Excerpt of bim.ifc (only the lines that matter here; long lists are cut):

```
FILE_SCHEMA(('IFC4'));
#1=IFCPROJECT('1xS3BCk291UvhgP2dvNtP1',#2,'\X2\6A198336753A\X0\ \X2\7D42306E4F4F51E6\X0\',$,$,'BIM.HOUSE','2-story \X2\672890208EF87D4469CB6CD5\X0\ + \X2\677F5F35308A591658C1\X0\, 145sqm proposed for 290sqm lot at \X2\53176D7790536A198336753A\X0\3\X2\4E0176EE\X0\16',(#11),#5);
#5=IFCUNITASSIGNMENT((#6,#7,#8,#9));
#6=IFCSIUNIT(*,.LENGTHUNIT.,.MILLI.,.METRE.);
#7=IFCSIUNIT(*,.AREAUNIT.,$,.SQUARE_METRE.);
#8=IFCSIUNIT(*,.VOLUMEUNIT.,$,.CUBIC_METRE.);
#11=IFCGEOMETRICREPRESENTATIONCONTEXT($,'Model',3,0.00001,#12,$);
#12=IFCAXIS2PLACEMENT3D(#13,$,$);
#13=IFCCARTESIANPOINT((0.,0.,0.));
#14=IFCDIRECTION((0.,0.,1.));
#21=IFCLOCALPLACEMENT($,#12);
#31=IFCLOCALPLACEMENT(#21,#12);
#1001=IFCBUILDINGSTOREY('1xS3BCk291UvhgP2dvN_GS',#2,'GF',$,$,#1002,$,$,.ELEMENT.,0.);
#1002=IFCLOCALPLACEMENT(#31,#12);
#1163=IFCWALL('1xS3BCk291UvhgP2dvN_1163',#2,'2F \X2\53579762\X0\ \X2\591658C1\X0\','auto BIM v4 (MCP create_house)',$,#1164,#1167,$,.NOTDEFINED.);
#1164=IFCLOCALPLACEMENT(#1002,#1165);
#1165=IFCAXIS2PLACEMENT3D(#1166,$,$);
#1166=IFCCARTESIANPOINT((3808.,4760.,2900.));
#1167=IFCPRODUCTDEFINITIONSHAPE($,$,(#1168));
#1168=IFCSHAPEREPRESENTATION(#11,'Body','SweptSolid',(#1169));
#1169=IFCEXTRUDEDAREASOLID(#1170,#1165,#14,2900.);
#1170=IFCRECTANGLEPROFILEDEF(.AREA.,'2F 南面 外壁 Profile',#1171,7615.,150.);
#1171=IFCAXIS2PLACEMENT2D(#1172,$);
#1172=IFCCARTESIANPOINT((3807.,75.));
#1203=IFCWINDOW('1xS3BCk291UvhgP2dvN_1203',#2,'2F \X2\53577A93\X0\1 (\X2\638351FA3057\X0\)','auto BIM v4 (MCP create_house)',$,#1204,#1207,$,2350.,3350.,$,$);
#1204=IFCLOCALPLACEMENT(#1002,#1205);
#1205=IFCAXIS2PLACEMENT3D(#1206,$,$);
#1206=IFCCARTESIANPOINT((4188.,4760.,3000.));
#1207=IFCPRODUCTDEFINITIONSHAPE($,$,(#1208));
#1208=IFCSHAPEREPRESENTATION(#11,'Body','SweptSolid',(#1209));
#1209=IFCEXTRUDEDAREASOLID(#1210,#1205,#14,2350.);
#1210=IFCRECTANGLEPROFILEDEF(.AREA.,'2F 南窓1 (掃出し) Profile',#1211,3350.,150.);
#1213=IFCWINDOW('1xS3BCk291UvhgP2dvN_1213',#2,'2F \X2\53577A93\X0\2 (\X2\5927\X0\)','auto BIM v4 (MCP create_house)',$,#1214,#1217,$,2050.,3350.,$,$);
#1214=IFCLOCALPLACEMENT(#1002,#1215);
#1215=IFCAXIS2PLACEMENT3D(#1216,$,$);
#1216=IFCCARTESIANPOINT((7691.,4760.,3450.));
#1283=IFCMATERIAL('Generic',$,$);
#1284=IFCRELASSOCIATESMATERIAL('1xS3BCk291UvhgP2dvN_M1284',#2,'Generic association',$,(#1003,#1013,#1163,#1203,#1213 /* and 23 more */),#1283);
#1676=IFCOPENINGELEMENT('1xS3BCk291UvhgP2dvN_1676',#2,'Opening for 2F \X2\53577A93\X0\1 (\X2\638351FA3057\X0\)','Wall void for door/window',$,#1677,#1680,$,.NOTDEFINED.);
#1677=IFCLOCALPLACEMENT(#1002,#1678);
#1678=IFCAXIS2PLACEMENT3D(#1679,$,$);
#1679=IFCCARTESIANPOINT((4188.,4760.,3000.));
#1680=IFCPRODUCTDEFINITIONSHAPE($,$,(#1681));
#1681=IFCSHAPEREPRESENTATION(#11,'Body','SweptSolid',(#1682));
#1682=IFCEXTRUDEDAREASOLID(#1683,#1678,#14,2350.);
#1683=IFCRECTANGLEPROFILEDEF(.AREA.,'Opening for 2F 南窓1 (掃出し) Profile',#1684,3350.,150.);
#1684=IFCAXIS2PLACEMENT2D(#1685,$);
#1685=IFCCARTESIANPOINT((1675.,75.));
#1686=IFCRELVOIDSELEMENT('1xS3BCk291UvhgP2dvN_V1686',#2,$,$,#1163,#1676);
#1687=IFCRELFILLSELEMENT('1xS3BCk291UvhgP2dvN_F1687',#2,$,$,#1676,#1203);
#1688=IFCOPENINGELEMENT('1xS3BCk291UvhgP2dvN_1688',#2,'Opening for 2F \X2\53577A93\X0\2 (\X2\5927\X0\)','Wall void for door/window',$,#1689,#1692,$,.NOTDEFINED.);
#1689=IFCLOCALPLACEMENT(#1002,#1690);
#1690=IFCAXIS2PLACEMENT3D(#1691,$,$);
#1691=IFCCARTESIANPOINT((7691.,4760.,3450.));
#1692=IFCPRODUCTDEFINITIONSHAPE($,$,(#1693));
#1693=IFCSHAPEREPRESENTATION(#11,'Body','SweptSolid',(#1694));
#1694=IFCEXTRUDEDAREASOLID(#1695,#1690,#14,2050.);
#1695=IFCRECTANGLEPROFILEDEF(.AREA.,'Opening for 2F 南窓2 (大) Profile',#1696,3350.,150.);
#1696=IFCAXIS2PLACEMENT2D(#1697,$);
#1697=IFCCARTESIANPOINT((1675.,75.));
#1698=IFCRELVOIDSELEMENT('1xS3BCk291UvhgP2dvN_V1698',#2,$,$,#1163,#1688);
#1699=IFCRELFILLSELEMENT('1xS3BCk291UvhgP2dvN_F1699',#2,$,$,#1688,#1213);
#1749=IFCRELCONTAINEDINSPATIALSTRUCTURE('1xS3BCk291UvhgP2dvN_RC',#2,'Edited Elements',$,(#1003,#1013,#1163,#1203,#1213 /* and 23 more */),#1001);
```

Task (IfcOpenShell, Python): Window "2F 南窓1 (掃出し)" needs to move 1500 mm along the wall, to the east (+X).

```python
import ifcopenshell
import ifcopenshell.api.geometry
import ifcopenshell.util.placement
import ifcopenshell.util.unit

model = ifcopenshell.open("bim.ifc")
unit_scale = ifcopenshell.util.unit.calculate_unit_scale(model)

window = model.by_guid("1xS3BCk291UvhgP2dvN_1203")
opening = window.FillsVoids[0].RelatingOpeningElement
wall = opening.VoidsElements[0].RelatingBuildingElement

wall_matrix = ifcopenshell.util.placement.get_local_placement(wall.ObjectPlacement)
shift = wall_matrix[:3, 0] * 1.5 / unit_scale
before = ifcopenshell.util.placement.get_local_placement(window.ObjectPlacement)[:3, 3].copy()

# The window is not placed relative to its opening, so move both.
for product in (opening, window):
    matrix = ifcopenshell.util.placement.get_local_placement(product.ObjectPlacement)
    matrix[:3, 3] += shift
    ifcopenshell.api.geometry.edit_object_placement(model, product=product, matrix=matrix, is_si=False)

after = ifcopenshell.util.placement.get_local_placement(window.ObjectPlacement)[:3, 3]
print("window moved by", (after - before).round(3) + 0.0)

model.write("bim_updated.ifc")
```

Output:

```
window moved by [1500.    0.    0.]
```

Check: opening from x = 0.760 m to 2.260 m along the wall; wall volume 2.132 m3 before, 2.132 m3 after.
